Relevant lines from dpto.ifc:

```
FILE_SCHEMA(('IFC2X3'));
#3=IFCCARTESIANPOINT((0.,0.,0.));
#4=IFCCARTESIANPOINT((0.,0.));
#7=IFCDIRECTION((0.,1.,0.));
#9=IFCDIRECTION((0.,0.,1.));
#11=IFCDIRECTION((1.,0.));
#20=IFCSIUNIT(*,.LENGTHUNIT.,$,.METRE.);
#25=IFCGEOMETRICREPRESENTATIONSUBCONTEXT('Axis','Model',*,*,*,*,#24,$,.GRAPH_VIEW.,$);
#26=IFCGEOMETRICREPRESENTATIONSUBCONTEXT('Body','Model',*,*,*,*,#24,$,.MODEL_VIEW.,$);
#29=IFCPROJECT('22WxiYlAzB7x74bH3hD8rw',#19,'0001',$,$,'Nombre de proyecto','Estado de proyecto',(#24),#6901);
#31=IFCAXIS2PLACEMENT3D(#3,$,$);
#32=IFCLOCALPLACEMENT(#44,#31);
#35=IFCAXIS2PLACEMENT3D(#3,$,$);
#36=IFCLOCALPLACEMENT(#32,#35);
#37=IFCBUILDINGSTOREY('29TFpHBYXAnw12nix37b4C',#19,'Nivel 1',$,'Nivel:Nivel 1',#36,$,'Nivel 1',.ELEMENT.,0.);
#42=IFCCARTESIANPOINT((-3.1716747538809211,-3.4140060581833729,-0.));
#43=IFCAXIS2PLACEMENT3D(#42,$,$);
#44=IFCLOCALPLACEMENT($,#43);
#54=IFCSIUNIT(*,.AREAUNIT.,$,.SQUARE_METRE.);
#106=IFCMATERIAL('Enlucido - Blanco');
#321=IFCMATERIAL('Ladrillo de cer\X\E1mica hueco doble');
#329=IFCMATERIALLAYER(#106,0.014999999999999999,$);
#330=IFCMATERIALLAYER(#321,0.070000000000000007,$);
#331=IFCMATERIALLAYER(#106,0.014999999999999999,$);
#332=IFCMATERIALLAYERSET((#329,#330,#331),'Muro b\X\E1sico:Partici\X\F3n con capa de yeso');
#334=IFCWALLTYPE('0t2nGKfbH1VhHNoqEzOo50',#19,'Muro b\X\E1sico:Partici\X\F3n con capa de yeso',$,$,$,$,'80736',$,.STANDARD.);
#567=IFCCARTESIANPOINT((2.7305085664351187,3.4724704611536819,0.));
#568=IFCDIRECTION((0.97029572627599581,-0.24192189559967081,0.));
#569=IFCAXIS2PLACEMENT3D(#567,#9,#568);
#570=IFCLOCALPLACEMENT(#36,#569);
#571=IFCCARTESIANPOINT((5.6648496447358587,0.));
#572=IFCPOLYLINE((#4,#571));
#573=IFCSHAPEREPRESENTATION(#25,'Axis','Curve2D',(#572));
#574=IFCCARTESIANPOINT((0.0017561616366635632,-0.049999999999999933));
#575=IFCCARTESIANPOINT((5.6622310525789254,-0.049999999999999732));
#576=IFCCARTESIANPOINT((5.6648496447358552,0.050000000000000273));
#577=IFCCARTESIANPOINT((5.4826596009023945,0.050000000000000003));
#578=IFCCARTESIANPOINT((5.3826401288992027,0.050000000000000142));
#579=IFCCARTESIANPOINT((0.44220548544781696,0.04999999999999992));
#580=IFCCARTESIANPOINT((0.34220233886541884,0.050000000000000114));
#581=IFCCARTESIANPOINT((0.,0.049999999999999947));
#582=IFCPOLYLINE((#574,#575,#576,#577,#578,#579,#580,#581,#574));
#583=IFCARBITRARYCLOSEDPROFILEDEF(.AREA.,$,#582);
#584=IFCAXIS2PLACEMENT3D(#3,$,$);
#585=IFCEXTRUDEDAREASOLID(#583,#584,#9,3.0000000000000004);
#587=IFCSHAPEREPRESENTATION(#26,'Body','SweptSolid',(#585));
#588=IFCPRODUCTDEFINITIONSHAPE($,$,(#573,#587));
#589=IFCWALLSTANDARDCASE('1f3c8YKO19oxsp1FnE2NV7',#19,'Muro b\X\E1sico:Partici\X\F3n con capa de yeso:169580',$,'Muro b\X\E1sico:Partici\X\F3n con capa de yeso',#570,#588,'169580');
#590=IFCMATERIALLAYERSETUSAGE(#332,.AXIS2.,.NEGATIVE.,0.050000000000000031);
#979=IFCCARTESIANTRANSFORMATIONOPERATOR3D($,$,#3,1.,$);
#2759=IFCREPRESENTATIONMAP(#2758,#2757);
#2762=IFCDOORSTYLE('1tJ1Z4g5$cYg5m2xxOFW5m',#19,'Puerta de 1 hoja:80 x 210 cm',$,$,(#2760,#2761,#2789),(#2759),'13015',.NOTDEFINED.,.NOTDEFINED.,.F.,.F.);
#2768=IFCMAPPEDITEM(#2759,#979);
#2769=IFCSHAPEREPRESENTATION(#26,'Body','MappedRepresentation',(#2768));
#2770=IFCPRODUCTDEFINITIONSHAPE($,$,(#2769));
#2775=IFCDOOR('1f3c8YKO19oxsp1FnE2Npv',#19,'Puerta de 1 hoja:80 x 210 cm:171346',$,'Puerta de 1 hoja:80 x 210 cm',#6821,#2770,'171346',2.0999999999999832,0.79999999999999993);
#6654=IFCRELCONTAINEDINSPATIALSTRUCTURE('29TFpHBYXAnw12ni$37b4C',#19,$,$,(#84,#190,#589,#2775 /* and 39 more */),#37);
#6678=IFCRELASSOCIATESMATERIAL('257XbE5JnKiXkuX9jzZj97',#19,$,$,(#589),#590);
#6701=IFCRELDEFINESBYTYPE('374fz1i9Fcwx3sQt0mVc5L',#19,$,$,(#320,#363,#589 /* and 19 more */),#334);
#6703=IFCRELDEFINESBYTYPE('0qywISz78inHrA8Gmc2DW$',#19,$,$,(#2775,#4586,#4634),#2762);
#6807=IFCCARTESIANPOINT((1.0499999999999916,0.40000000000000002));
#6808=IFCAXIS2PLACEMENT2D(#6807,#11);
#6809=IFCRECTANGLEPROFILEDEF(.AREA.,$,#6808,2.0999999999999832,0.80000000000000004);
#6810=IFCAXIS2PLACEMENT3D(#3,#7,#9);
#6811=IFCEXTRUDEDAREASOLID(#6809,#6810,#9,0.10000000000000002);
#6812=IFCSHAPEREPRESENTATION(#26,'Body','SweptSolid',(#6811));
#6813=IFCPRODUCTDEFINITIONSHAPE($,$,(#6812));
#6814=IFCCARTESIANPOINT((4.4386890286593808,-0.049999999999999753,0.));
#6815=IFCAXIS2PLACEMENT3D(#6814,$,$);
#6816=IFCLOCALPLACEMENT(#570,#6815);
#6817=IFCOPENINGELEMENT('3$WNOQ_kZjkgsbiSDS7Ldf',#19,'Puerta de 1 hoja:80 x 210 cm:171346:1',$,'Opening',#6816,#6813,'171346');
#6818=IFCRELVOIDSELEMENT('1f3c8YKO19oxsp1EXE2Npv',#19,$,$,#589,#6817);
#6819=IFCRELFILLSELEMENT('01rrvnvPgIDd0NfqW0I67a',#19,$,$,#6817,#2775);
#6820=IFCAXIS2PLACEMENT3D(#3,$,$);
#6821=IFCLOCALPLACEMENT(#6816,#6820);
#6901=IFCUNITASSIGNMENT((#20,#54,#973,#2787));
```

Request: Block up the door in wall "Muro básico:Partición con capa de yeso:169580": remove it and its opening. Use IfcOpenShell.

```python
import ifcopenshell
import ifcopenshell.api.feature
import ifcopenshell.api.root
import ifcopenshell.geom
import ifcopenshell.util.shape

model = ifcopenshell.open("dpto.ifc")
settings = ifcopenshell.geom.settings()


def volume(element):
    """Net volume in cubic metres, openings subtracted."""
    shape = ifcopenshell.geom.create_shape(settings, element)
    return ifcopenshell.util.shape.get_volume(shape.geometry)


door = model.by_guid("1f3c8YKO19oxsp1FnE2Npv")
opening = door.FillsVoids[0].RelatingOpeningElement
wall = opening.VoidsElements[0].RelatingBuildingElement
before = volume(wall)

ifcopenshell.api.root.remove_product(model, product=door)
ifcopenshell.api.feature.remove_feature(model, feature=opening)

after = volume(wall)

print(f"wall volume {before:.3f} -> {after:.3f} m3")

model.write("dpto_rev.ifc")
```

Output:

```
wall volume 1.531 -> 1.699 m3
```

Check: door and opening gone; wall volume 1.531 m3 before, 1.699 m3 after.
